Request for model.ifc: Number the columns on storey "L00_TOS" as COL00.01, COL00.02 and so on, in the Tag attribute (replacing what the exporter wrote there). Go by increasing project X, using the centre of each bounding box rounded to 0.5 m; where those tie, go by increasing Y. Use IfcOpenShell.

First a look at what the model holds.

```python
import ifcopenshell
import ifcopenshell.util.element
import ifcopenshell.util.placement

model = ifcopenshell.open("model.ifc")
print(model.schema)
storey = next(s for s in model.by_type("IfcBuildingStorey") if s.Name == "L00_TOS")
columns = [e for e in ifcopenshell.util.element.get_decomposition(storey) if e.is_a("IfcColumn")]
for e in sorted(columns, key=lambda e: e.id()):
    origin = ifcopenshell.util.placement.get_local_placement(e.ObjectPlacement)[:3, 3]
    print(e.id(), e.Tag, e.Name, origin.round(2) + 0.0, sep=" | ")
```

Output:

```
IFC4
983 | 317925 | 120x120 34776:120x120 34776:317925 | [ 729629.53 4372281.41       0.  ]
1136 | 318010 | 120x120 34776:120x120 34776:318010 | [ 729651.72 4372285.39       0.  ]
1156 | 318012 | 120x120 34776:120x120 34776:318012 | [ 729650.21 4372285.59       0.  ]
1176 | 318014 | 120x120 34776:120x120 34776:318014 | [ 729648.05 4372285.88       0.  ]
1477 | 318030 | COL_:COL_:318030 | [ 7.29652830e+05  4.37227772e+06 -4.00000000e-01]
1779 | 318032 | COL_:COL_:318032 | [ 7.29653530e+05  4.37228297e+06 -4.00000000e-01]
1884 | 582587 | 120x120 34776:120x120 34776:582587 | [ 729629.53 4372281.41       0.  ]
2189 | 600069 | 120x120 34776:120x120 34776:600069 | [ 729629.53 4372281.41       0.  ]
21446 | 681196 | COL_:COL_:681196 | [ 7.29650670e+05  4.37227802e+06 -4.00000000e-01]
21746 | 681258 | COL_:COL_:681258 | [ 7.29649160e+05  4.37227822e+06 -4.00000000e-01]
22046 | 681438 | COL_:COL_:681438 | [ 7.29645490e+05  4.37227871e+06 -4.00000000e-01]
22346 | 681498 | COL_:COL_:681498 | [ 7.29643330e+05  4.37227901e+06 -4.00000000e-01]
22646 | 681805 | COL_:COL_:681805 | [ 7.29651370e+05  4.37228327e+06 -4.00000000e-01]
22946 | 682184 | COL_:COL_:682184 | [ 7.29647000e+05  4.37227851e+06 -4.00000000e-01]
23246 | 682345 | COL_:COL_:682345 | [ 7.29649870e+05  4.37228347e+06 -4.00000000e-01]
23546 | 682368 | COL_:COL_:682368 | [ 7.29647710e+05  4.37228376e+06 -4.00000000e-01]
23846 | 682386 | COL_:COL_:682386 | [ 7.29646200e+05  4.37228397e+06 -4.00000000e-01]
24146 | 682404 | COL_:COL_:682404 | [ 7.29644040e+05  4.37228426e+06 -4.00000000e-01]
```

```python
import ifcopenshell
import ifcopenshell.geom
import ifcopenshell.util.element
import ifcopenshell.util.shape

model = ifcopenshell.open("model.ifc")
settings = ifcopenshell.geom.settings()
settings.set("use-world-coords", True)


def centre(element):
    shape = ifcopenshell.geom.create_shape(settings, element)
    return ifcopenshell.util.shape.get_bbox_centroid(shape.geometry)


storey = next(s for s in model.by_type("IfcBuildingStorey") if s.Name == "L00_TOS")
columns = [e for e in ifcopenshell.util.element.get_decomposition(storey) if e.is_a("IfcColumn")]

# Insertion points can sit at a corner or the storey origin, so sort by the geometry (in metres).
centres = {e: centre(e) for e in columns}
columns.sort(key=lambda e: (round(centres[e][0] / 0.5), centres[e][1]))

for i, e in enumerate(columns, start=1):
    number = f"COL00.{i:02d}"
    e.Tag = number
    print(e.id(), number)

model.write("model-out.ifc")
```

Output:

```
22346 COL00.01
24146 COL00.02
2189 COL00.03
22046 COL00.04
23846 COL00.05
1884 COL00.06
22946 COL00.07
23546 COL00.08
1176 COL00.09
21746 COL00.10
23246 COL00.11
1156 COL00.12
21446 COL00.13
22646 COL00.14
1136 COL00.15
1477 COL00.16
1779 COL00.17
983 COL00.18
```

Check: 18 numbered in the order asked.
